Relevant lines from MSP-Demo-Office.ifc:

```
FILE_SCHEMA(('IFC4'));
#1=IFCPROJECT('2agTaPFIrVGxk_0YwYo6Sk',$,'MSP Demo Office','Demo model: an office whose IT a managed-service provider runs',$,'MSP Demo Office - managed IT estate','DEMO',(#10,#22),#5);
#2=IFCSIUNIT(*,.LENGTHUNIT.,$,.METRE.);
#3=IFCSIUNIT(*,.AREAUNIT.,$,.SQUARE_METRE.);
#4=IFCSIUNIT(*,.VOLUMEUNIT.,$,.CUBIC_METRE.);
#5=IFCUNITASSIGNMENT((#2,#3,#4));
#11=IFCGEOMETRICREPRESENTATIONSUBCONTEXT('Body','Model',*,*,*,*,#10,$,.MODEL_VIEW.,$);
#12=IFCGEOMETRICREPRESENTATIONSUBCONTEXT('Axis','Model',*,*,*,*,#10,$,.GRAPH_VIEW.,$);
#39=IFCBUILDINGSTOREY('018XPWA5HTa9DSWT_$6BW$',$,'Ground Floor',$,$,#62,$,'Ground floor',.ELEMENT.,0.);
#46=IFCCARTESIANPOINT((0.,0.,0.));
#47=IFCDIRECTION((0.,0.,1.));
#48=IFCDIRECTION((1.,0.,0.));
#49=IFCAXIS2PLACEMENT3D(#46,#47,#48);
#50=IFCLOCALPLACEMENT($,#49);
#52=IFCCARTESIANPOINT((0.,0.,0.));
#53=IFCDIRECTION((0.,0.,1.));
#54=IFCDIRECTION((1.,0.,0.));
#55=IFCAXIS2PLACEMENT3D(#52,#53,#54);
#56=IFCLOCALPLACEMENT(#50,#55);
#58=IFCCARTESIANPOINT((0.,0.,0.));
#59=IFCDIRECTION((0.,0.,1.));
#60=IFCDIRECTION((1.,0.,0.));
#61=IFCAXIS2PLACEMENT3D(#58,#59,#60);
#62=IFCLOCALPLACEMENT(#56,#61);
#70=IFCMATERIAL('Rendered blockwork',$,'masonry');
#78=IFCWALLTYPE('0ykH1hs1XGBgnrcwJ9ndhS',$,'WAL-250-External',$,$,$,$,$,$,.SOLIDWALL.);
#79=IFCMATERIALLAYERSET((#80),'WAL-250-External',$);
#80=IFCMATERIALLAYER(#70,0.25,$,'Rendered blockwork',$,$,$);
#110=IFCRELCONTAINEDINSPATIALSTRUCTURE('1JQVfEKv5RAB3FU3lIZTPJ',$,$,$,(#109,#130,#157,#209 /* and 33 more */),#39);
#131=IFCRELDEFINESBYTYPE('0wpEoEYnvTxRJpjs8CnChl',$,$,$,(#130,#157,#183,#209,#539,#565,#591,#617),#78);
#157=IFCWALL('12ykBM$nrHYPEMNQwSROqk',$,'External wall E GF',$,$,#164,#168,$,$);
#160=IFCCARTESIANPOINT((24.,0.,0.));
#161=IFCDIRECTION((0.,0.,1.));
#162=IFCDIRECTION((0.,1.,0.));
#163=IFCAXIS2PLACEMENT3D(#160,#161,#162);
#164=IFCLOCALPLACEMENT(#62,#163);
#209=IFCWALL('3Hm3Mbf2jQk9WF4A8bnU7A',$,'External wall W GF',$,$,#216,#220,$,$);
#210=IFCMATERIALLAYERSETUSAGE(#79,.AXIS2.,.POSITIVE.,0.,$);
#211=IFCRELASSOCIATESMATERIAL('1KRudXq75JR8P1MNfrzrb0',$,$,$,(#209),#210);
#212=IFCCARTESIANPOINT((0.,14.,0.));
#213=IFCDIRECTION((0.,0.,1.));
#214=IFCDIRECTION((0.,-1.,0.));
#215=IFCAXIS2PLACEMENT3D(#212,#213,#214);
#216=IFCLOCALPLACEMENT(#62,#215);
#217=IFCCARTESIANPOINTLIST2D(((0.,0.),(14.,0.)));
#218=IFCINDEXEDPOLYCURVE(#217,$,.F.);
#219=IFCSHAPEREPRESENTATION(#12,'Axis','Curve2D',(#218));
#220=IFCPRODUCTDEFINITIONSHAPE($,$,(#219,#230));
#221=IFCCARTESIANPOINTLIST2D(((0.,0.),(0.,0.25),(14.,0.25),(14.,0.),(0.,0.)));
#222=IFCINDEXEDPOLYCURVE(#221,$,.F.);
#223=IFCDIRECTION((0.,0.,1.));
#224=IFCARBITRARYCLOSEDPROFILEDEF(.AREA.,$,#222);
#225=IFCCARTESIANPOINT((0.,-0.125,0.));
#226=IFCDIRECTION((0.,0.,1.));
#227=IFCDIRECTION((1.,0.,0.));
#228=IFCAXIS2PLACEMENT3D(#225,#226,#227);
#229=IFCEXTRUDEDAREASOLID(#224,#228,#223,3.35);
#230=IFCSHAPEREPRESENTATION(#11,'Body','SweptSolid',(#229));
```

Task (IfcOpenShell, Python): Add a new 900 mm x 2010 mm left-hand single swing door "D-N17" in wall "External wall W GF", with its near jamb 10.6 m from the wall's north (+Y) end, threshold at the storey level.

```python
import numpy as np
import ifcopenshell
import ifcopenshell.api.feature
import ifcopenshell.api.geometry
import ifcopenshell.api.root
import ifcopenshell.api.spatial
import ifcopenshell.geom
import ifcopenshell.util.element
import ifcopenshell.util.placement
import ifcopenshell.util.representation
import ifcopenshell.util.shape
import ifcopenshell.util.unit

model = ifcopenshell.open("MSP-Demo-Office.ifc")
unit_scale = ifcopenshell.util.unit.calculate_unit_scale(model)
settings = ifcopenshell.geom.settings()


def volume(element):
    """Net volume in cubic metres, openings subtracted."""
    shape = ifcopenshell.geom.create_shape(settings, element)
    return ifcopenshell.util.shape.get_volume(shape.geometry)


wall = model.by_guid("3Hm3Mbf2jQk9WF4A8bnU7A")
storey = ifcopenshell.util.element.get_container(wall, ifc_class="IfcBuildingStorey")
context = ifcopenshell.util.representation.get_context(model, "Model", "Body", "MODEL_VIEW")
before = volume(wall)

width, height, from_end, sill = 0.9, 2.01, 10.6, 0.0  # metres

# The wall runs along its own X axis, and the end named is its -X end.
wall_shape = ifcopenshell.geom.create_shape(settings, wall)
x, y, z = ifcopenshell.util.shape.get_vertices(wall_shape.geometry).T
start = x.min() + from_end
face, thickness = float(y.min()), float(y.max() - y.min())
wall_matrix = ifcopenshell.util.placement.get_local_placement(wall.ObjectPlacement)
level = ifcopenshell.util.placement.get_local_placement(storey.ObjectPlacement)[2, 3]


def in_wall(x, y):
    """Placement at x, y metres in the wall's axes, at sill height."""
    matrix = wall_matrix.copy()
    matrix[:, 3] = wall_matrix @ np.array([x / unit_scale, y / unit_scale, 0.0, 1.0])
    matrix[2, 3] = level + sill / unit_scale
    return matrix


# Opening: a box that overshoots both wall faces by 50 mm.
opening = ifcopenshell.api.root.create_entity(model, ifc_class="IfcOpeningElement", predefined_type="OPENING")
box = ifcopenshell.api.geometry.add_wall_representation(
    model, context=context, length=width, height=height, thickness=thickness + 0.1
)
ifcopenshell.api.geometry.assign_representation(model, product=opening, representation=box)
ifcopenshell.api.geometry.edit_object_placement(model, product=opening, matrix=in_wall(start, face - 0.05), is_si=False)
ifcopenshell.api.feature.add_feature(model, feature=opening, element=wall)

door = ifcopenshell.api.root.create_entity(model, ifc_class="IfcDoor", name="D-N17", predefined_type="DOOR")
door.OverallWidth, door.OverallHeight = width / unit_scale, height / unit_scale
door.OperationType = "SINGLE_SWING_LEFT"
body = ifcopenshell.api.geometry.add_door_representation(
    model,
    context=context,
    overall_width=door.OverallWidth,
    overall_height=door.OverallHeight,
    operation_type="SINGLE_SWING_LEFT",
    lining_properties={"LiningDepth": thickness / unit_scale, "ThresholdDepth": thickness / unit_scale},
)
ifcopenshell.api.geometry.assign_representation(model, product=door, representation=body)
ifcopenshell.api.spatial.assign_container(model, products=[door], relating_structure=storey)
ifcopenshell.api.feature.add_filling(model, opening=opening, element=door)

# The lining spans the wall, so the door starts at the wall face.
ifcopenshell.api.geometry.edit_object_placement(model, product=door, matrix=in_wall(start, face), is_si=False)

after = volume(wall)

print(f"wall volume {before:.3f} -> {after:.3f} m3")

model.write("MSP-Demo-Office_rev.ifc")
```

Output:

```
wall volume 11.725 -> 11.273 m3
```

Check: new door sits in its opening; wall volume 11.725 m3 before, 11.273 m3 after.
